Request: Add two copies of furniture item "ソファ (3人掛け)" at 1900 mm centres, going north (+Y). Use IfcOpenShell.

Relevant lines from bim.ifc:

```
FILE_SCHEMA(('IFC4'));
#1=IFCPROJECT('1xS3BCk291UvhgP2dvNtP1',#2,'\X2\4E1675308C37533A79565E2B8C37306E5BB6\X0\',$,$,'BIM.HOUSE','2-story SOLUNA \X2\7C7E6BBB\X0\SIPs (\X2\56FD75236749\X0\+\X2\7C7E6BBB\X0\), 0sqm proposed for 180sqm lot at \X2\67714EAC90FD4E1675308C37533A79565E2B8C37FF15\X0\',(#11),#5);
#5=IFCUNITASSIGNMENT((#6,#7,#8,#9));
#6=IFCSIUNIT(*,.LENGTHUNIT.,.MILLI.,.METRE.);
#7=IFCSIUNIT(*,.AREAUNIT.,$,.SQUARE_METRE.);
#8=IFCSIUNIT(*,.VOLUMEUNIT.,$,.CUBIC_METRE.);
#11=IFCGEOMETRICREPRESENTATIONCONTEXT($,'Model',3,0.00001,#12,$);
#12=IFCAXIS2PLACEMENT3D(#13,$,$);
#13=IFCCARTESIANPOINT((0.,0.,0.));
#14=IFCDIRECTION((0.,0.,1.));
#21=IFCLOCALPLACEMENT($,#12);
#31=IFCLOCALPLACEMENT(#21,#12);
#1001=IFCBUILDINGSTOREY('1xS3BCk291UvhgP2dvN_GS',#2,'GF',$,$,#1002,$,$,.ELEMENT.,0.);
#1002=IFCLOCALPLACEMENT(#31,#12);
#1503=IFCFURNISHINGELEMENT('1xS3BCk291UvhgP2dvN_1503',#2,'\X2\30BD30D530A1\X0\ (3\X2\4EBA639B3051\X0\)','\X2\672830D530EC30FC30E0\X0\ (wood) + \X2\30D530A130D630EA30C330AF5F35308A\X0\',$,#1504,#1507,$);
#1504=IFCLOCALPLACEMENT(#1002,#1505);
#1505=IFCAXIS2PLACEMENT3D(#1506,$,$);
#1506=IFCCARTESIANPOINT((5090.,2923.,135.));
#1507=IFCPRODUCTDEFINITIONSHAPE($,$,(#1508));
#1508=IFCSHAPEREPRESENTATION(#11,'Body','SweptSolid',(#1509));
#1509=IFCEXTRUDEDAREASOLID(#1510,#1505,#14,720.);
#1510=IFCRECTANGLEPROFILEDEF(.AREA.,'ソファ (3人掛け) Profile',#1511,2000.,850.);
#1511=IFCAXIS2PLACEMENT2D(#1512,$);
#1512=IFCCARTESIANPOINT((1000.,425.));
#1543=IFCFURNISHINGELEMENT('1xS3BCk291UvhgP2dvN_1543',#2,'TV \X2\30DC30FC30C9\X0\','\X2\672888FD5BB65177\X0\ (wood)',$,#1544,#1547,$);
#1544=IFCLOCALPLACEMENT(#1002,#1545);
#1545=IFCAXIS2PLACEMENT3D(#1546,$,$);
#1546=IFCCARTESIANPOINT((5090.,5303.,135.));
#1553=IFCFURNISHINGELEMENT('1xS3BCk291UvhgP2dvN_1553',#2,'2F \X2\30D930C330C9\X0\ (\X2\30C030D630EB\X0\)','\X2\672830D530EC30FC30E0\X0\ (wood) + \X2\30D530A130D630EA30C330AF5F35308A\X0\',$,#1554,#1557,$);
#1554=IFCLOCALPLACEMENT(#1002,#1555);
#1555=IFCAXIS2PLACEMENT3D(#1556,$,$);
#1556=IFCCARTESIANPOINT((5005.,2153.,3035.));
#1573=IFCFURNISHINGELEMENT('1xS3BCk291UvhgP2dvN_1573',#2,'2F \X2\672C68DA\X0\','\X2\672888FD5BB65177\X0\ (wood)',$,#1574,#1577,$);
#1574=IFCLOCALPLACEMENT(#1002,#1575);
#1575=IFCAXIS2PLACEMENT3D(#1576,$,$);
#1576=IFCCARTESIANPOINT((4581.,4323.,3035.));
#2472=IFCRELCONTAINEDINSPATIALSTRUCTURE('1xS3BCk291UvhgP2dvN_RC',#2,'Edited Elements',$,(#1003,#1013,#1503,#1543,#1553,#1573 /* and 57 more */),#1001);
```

```python
import numpy as np
import ifcopenshell
import ifcopenshell.api.geometry
import ifcopenshell.api.root
import ifcopenshell.util.element
import ifcopenshell.util.placement
import ifcopenshell.util.unit

model = ifcopenshell.open("bim.ifc")
unit_scale = ifcopenshell.util.unit.calculate_unit_scale(model)


def reuse_history(source, copy):
    """copy_class also copies each property set's owner history, people and application; keep the originals."""
    for rel in copy.IsDefinedBy:
        if rel.is_a("IfcRelDefinesByProperties") and (history := rel.RelatingPropertyDefinition.OwnerHistory):
            rel.RelatingPropertyDefinition.OwnerHistory = source.OwnerHistory
            ifcopenshell.util.element.remove_deep2(model, history)


source = model.by_guid("1xS3BCk291UvhgP2dvN_1503")
base = ifcopenshell.util.placement.get_local_placement(source.ObjectPlacement)
step = np.array([0.0, 1.0, 0.0]) * 1.9 / unit_scale

for i in range(1, 3):
    copy = ifcopenshell.api.root.copy_class(model, product=source)
    copy.Representation = ifcopenshell.util.element.copy_deep(
        model, source.Representation, exclude=["IfcGeometricRepresentationContext", "IfcRepresentationMap"]
    )
    reuse_history(source, copy)
    matrix = base.copy()
    matrix[:3, 3] += i * step
    print("added at", matrix[:3, 3].round(3) + 0.0)
    ifcopenshell.api.geometry.edit_object_placement(model, product=copy, matrix=matrix, is_si=False)

model.write("bim-out.ifc")
```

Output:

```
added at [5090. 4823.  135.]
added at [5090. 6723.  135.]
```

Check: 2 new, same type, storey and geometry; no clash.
